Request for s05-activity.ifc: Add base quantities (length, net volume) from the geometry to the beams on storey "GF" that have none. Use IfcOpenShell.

First a look at what the model holds.

```python
import ifcopenshell
import ifcopenshell.util.element
import ifcopenshell.util.unit

model = ifcopenshell.open("s05-activity.ifc")
print(model.schema)
for unit_type in ("LENGTHUNIT", "AREAUNIT", "VOLUMEUNIT"):
    print(unit_type, ifcopenshell.util.unit.calculate_unit_scale(model, unit_type))
storey = next(s for s in model.by_type("IfcBuildingStorey") if s.Name == "GF")
beams = [e for e in ifcopenshell.util.element.get_decomposition(storey) if e.is_a("IfcBeam")]
for e in sorted(beams, key=lambda e: e.id()):
    print(e.id(), e.is_a(), e.Name, list(ifcopenshell.util.element.get_psets(e, qtos_only=True)), sep=" | ")
```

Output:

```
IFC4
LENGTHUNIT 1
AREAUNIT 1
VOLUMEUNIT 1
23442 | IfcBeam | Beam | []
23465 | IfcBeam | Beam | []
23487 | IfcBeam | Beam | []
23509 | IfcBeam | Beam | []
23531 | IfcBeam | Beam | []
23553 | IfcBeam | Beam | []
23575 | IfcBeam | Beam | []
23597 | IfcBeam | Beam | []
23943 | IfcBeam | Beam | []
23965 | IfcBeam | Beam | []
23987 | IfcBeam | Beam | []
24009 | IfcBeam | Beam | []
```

```python
import ifcopenshell
import ifcopenshell.api.pset
import ifcopenshell.geom
import ifcopenshell.util.element
import ifcopenshell.util.shape
import ifcopenshell.util.unit

model = ifcopenshell.open("s05-activity.ifc")
unit_scale = ifcopenshell.util.unit.calculate_unit_scale(model)
volume_scale = ifcopenshell.util.unit.calculate_unit_scale(model, "VOLUMEUNIT")
settings = ifcopenshell.geom.settings()

storey = next(s for s in model.by_type("IfcBuildingStorey") if s.Name == "GF")
beams = [e for e in ifcopenshell.util.element.get_decomposition(storey) if e.is_a("IfcBeam")]

for e in sorted(beams, key=lambda e: e.id()):
    if ifcopenshell.util.element.get_psets(e, qtos_only=True, should_inherit=False):
        continue
    # Geometry comes back in metres, in the element's own axes.
    shape = ifcopenshell.geom.create_shape(settings, e)
    values = {
        "Length": ifcopenshell.util.shape.get_max_xyz(shape.geometry) / unit_scale,
        "NetVolume": ifcopenshell.util.shape.get_volume(shape.geometry) / volume_scale,
    }
    qto = ifcopenshell.api.pset.add_qto(model, product=e, name="Qto_BeamBaseQuantities")
    ifcopenshell.api.pset.edit_qto(model, qto=qto, properties=values)
    print(e.id(), {k: round(v, 3) for k, v in values.items()})

model.write("s05-activity_rev.ifc")
```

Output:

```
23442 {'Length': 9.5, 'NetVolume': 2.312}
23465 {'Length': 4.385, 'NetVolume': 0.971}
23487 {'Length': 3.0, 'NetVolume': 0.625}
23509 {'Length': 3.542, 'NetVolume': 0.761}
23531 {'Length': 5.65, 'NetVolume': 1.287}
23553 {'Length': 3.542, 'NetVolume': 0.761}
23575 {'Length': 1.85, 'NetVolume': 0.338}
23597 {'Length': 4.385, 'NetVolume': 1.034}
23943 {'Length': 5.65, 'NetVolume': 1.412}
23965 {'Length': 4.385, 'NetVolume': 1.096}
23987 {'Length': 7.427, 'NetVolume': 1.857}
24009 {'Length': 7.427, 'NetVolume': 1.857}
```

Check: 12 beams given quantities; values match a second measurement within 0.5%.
